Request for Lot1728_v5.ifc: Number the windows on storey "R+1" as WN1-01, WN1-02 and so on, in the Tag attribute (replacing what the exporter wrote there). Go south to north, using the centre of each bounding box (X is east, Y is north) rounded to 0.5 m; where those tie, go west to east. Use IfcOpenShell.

First a look at what the model holds.

```python
import ifcopenshell
import ifcopenshell.util.element
import ifcopenshell.util.placement

model = ifcopenshell.open("Lot1728_v5.ifc")
print(model.schema)
storey = next(s for s in model.by_type("IfcBuildingStorey") if s.Name == "R+1")
windows = [e for e in ifcopenshell.util.element.get_decomposition(storey) if e.is_a("IfcWindow")]
for e in sorted(windows, key=lambda e: e.id()):
    origin = ifcopenshell.util.placement.get_local_placement(e.ObjectPlacement)[:3, 3]
    print(e.id(), e.Tag, e.Name, origin.round(2) + 0.0, sep=" | ")
```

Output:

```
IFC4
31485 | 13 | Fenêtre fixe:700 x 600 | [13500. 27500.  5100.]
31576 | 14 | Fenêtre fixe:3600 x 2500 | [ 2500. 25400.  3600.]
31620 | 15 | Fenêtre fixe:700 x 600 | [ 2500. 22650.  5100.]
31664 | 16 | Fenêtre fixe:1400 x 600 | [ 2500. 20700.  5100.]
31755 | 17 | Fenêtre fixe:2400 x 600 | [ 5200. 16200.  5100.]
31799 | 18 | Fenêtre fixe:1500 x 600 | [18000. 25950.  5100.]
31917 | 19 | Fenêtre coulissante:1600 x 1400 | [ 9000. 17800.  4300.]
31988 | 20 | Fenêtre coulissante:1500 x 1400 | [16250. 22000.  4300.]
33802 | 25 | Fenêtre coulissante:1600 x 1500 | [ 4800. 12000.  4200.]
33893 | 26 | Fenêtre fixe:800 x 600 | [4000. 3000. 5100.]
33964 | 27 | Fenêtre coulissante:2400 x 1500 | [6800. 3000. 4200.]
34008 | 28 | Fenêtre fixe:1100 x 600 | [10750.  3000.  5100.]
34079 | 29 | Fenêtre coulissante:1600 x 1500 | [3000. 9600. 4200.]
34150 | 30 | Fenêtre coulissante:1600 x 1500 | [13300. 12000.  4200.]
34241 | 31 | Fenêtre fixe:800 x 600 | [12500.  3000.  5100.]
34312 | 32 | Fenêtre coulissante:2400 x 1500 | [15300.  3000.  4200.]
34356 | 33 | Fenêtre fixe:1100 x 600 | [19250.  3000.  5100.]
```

```python
import ifcopenshell
import ifcopenshell.geom
import ifcopenshell.util.element
import ifcopenshell.util.shape

model = ifcopenshell.open("Lot1728_v5.ifc")
settings = ifcopenshell.geom.settings()
settings.set("use-world-coords", True)


def centre(element):
    shape = ifcopenshell.geom.create_shape(settings, element)
    return ifcopenshell.util.shape.get_bbox_centroid(shape.geometry)


storey = next(s for s in model.by_type("IfcBuildingStorey") if s.Name == "R+1")
windows = [e for e in ifcopenshell.util.element.get_decomposition(storey) if e.is_a("IfcWindow")]

# Insertion points can sit at a corner or the storey origin, so sort by the geometry (in metres).
centres = {e: centre(e) for e in windows}
windows.sort(key=lambda e: (round(centres[e][1] / 0.5), centres[e][0]))

for i, e in enumerate(windows, start=1):
    number = f"WN1-{i:02d}"
    e.Tag = number
    print(e.id(), number)

model.write("Lot1728_v5_updated.ifc")
```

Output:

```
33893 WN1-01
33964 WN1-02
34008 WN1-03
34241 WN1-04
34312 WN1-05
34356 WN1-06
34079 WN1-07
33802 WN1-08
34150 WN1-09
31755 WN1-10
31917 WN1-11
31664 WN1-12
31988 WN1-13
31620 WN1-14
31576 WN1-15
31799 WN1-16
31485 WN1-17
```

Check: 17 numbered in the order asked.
